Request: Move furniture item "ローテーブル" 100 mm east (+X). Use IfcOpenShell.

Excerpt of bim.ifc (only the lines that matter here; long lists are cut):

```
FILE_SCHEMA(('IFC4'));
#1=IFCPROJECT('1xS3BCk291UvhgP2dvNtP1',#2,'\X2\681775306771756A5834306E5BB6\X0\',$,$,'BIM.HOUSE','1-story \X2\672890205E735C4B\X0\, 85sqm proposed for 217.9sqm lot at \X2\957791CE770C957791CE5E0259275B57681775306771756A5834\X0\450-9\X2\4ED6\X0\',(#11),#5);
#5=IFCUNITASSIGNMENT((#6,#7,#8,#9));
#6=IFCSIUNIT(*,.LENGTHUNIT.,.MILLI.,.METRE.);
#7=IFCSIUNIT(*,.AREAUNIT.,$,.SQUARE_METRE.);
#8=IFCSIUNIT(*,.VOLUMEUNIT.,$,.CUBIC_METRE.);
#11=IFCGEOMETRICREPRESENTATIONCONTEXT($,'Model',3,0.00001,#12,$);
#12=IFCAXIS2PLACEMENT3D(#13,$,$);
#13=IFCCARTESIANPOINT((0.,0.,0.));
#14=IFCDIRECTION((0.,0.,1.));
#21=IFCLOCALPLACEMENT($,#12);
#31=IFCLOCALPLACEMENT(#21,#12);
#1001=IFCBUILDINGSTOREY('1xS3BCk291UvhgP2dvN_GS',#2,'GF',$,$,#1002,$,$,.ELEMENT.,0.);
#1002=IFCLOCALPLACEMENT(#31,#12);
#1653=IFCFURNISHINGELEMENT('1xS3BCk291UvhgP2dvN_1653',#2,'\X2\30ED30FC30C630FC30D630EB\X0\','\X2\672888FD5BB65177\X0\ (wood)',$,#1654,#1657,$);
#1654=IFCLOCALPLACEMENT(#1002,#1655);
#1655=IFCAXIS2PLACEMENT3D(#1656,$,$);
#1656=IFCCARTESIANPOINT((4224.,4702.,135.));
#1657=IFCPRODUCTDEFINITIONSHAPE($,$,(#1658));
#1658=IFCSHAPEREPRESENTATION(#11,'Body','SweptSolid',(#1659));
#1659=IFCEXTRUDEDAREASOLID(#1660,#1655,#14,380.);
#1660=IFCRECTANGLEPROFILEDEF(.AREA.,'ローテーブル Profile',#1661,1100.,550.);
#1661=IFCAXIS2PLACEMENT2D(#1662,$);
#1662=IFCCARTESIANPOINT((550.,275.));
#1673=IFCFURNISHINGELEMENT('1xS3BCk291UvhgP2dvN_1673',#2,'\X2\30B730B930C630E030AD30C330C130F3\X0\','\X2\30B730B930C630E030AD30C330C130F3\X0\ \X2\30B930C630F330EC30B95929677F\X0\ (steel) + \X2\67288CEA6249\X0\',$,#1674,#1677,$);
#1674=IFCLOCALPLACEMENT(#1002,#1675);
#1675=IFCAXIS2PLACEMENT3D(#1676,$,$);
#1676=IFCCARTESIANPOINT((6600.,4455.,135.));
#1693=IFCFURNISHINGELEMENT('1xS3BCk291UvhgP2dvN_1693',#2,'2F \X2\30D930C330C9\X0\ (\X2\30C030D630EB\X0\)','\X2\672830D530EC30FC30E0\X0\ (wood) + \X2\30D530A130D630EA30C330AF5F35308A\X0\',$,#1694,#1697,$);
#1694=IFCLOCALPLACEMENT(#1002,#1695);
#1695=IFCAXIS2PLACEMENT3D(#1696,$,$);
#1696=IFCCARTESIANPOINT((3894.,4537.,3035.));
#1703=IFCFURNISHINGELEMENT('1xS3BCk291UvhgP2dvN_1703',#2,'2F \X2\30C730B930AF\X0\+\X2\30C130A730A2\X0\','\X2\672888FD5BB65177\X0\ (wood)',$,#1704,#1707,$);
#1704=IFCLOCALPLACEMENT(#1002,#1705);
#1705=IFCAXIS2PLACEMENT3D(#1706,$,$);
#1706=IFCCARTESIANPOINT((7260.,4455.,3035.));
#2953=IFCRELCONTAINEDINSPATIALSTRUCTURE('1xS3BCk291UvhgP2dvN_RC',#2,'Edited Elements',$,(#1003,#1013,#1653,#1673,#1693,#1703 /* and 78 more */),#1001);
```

```python
import ifcopenshell
import ifcopenshell.api.geometry
import ifcopenshell.util.placement

model = ifcopenshell.open("bim.ifc")

item = model.by_guid("1xS3BCk291UvhgP2dvN_1653")
matrix = ifcopenshell.util.placement.get_local_placement(item.ObjectPlacement)
matrix[0, 3] += 100.0
ifcopenshell.api.geometry.edit_object_placement(model, product=item, matrix=matrix, is_si=False)

print(ifcopenshell.util.placement.get_local_placement(item.ObjectPlacement).round(3) + 0.0)

model.write("bim_rev.ifc")
```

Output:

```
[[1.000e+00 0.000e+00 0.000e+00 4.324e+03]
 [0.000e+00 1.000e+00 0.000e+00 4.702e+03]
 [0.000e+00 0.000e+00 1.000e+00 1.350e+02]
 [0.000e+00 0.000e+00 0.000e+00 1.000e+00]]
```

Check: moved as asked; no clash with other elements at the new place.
